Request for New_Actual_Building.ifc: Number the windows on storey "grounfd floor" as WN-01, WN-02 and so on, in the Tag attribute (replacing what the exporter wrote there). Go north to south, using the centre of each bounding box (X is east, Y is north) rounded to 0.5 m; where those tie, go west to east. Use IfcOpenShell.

First a look at what the model holds.

```python
import ifcopenshell
import ifcopenshell.util.element
import ifcopenshell.util.placement

model = ifcopenshell.open("New_Actual_Building.ifc")
print(model.schema)
storey = next(s for s in model.by_type("IfcBuildingStorey") if s.Name == "grounfd floor")
windows = [e for e in ifcopenshell.util.element.get_decomposition(storey) if e.is_a("IfcWindow")]
for e in sorted(windows, key=lambda e: e.id()):
    origin = ifcopenshell.util.placement.get_local_placement(e.ObjectPlacement)[:3, 3]
    print(e.id(), e.Tag, e.Name, origin.round(2) + 0.0, sep=" | ")
```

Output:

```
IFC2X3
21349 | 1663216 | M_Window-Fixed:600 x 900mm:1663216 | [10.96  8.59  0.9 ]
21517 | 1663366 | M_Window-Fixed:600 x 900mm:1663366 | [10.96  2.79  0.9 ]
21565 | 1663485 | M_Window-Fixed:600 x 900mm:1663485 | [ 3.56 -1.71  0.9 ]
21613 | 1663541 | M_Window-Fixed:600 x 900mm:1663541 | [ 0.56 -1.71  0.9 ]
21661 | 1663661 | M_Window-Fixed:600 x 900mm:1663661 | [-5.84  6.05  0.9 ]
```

```python
import ifcopenshell
import ifcopenshell.geom
import ifcopenshell.util.element
import ifcopenshell.util.shape

model = ifcopenshell.open("New_Actual_Building.ifc")
settings = ifcopenshell.geom.settings()
settings.set("use-world-coords", True)


def centre(element):
    shape = ifcopenshell.geom.create_shape(settings, element)
    return ifcopenshell.util.shape.get_bbox_centroid(shape.geometry)


storey = next(s for s in model.by_type("IfcBuildingStorey") if s.Name == "grounfd floor")
windows = [e for e in ifcopenshell.util.element.get_decomposition(storey) if e.is_a("IfcWindow")]

# Insertion points can sit at a corner or the storey origin, so sort by the geometry (in metres).
centres = {e: centre(e) for e in windows}
windows.sort(key=lambda e: (-round(centres[e][1] / 0.5), centres[e][0]))

for i, e in enumerate(windows, start=1):
    number = f"WN-{i:02d}"
    e.Tag = number
    print(e.id(), number)

model.write("New_Actual_Building_edited.ifc")
```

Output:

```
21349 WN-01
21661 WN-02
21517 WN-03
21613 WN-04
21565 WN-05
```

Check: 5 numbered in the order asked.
